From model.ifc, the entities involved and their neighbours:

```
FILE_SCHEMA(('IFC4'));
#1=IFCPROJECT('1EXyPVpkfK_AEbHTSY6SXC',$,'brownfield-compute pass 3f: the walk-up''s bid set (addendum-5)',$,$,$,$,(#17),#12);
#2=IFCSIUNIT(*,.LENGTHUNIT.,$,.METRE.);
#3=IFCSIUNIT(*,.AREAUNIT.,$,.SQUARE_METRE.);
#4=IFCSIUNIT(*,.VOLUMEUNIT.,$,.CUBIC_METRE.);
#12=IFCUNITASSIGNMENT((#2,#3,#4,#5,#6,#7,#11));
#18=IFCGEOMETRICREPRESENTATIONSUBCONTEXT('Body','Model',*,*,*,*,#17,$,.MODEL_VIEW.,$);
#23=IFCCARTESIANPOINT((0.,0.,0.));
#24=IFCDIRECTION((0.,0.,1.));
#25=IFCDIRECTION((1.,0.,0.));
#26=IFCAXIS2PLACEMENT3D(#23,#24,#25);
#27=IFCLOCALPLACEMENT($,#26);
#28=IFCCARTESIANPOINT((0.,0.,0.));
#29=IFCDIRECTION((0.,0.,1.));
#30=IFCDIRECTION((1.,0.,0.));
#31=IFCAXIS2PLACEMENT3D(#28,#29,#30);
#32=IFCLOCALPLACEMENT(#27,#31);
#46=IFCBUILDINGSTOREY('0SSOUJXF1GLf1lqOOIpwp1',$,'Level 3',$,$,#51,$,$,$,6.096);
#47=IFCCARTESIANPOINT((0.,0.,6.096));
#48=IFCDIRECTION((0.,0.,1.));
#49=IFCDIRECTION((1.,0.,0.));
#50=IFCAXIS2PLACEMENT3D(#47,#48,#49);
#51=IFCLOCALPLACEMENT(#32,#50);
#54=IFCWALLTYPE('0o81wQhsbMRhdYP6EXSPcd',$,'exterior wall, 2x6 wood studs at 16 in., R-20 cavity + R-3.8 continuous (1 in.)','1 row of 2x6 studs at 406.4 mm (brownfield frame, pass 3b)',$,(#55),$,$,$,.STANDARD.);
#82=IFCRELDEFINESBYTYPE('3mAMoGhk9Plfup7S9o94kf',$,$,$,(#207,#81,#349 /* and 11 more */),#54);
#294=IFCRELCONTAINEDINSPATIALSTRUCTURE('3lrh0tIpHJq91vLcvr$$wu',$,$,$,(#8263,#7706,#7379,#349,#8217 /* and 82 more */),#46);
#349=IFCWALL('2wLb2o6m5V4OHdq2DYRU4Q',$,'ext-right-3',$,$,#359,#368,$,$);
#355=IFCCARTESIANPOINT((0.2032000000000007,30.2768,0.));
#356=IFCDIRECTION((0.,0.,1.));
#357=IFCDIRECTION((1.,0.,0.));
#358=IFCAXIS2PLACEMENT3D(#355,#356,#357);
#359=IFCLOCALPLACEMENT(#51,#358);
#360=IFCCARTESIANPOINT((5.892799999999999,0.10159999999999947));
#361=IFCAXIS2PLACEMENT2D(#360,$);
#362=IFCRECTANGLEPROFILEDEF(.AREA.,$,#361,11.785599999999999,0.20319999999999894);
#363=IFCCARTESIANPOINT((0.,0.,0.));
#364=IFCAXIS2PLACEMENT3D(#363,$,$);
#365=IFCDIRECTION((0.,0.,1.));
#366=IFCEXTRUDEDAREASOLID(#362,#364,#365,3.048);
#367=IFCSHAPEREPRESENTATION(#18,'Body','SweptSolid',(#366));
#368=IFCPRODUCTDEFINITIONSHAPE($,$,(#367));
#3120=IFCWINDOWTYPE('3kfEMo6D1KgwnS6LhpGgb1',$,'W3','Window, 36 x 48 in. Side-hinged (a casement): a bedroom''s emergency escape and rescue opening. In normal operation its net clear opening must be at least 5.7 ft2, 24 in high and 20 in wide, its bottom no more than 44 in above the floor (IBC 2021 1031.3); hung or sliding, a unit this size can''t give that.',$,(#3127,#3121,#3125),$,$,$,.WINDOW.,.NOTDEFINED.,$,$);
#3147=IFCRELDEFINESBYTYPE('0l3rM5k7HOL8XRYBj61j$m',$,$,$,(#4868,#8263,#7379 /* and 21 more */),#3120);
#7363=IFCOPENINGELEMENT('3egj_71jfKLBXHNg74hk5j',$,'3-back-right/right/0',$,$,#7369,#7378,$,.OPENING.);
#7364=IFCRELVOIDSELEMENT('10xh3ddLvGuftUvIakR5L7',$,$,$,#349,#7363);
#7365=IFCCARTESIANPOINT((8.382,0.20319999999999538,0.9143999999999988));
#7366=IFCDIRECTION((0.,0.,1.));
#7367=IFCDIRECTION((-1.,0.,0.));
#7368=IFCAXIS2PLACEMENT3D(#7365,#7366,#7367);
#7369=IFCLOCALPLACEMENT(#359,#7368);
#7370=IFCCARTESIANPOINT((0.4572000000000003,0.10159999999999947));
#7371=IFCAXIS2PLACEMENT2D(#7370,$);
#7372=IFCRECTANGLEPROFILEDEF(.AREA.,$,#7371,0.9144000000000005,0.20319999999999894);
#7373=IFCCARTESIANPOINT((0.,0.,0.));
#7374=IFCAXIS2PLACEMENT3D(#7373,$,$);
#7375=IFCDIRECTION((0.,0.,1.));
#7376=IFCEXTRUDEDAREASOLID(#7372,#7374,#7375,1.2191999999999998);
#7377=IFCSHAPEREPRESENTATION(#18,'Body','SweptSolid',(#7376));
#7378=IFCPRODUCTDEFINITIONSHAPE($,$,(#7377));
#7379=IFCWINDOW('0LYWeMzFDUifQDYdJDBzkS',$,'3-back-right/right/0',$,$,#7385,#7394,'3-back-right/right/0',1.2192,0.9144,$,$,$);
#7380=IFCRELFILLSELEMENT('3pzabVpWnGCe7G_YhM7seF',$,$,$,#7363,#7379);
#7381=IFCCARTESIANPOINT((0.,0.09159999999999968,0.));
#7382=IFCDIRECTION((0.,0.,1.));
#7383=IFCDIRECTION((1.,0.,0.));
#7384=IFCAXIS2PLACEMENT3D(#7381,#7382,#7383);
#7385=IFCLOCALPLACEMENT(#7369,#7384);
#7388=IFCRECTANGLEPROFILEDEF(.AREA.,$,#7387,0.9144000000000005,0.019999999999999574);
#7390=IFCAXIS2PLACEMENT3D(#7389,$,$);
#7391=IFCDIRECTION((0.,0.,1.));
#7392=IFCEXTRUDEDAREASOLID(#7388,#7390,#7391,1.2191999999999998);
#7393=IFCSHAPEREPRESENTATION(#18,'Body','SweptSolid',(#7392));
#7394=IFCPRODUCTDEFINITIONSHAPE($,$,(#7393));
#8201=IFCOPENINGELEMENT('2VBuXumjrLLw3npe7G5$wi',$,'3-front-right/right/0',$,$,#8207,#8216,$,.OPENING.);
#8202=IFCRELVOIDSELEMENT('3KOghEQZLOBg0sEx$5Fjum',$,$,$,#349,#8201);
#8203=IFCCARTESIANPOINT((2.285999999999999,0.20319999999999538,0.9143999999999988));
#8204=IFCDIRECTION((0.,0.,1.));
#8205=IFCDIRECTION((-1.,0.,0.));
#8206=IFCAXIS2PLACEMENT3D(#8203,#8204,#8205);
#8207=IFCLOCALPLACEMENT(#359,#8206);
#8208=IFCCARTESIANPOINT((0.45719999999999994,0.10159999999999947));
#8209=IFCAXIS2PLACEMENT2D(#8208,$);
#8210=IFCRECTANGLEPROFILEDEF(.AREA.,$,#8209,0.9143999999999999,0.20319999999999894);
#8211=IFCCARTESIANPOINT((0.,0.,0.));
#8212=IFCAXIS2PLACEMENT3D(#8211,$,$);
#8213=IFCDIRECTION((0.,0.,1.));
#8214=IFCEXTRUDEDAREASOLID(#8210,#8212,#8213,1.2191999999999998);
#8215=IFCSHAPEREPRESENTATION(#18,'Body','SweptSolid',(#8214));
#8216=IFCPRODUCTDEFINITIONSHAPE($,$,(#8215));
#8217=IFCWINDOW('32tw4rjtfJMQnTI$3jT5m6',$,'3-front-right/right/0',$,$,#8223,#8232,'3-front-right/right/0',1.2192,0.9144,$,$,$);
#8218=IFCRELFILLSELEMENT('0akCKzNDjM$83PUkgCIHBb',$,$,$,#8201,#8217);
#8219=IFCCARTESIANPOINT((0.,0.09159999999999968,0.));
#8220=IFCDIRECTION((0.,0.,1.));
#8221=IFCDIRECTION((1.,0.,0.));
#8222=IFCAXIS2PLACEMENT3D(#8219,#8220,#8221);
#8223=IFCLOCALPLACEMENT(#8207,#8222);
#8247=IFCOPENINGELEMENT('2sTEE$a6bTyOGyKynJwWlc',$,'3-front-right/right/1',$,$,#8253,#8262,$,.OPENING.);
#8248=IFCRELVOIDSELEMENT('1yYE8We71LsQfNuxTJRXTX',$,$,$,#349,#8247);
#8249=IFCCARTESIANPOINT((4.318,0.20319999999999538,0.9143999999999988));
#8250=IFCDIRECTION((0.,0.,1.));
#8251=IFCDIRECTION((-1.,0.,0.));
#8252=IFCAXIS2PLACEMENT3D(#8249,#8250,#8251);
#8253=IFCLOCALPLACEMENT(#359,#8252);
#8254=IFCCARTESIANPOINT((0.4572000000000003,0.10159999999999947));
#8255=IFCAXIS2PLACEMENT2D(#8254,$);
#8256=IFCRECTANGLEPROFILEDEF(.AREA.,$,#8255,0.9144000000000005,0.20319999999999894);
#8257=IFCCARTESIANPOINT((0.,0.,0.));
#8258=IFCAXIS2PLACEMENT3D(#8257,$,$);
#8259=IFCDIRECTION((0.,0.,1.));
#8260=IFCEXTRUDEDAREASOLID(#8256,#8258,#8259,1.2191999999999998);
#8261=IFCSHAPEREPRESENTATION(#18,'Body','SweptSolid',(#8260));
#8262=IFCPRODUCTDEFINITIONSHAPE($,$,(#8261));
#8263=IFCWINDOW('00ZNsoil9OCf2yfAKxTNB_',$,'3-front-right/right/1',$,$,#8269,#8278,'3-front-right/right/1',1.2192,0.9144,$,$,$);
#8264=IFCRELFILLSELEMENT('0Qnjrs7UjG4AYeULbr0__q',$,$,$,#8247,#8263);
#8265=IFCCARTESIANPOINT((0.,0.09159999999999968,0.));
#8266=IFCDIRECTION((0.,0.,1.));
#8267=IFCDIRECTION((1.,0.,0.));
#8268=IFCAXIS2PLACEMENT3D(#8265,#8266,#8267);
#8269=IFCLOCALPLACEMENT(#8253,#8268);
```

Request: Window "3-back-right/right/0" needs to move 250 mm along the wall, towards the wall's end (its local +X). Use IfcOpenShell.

```python
import ifcopenshell
import ifcopenshell.api.geometry
import ifcopenshell.util.placement
import ifcopenshell.util.unit

model = ifcopenshell.open("model.ifc")
unit_scale = ifcopenshell.util.unit.calculate_unit_scale(model)

window = model.by_guid("0LYWeMzFDUifQDYdJDBzkS")
opening = window.FillsVoids[0].RelatingOpeningElement
wall = opening.VoidsElements[0].RelatingBuildingElement

wall_matrix = ifcopenshell.util.placement.get_local_placement(wall.ObjectPlacement)
shift = wall_matrix[:3, 0] * 0.25 / unit_scale
before = ifcopenshell.util.placement.get_local_placement(window.ObjectPlacement)[:3, 3].copy()

# The window is placed relative to its opening, so it follows when the opening moves.
matrix = ifcopenshell.util.placement.get_local_placement(opening.ObjectPlacement)
matrix[:3, 3] += shift
ifcopenshell.api.geometry.edit_object_placement(
    model, product=opening, matrix=matrix, is_si=False, should_transform_children=True
)

after = ifcopenshell.util.placement.get_local_placement(window.ObjectPlacement)[:3, 3]
print("window moved by", (after - before).round(3) + 0.0)

model.write("model-out.ifc")
```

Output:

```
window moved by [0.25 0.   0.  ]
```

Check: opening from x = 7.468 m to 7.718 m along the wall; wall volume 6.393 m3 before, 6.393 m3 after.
